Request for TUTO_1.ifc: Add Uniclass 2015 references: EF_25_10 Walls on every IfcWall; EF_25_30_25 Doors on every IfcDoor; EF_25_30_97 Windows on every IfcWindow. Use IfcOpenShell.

First a look at what the model holds.

```python
import ifcopenshell

model = ifcopenshell.open("TUTO_1.ifc")
print(model.schema)
print("classifications:", [c.Name for c in model.by_type("IfcClassification")])
for ifc_class in ("IfcDoor", "IfcRoof", "IfcStair", "IfcWall", "IfcWindow"):
    print(ifc_class, len(model.by_type(ifc_class)))
```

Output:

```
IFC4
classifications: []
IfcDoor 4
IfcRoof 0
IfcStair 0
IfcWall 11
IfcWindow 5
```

```python
import ifcopenshell
import ifcopenshell.api.classification

model = ifcopenshell.open("TUTO_1.ifc")

system = ifcopenshell.api.classification.add_classification(model, classification="Uniclass 2015")

codes = {
    "IfcWall": ("EF_25_10", "Walls"),
    "IfcDoor": ("EF_25_30_25", "Doors"),
    "IfcWindow": ("EF_25_30_97", "Windows"),
}
for ifc_class, (code, name) in codes.items():
    products = model.by_type(ifc_class)
    ifcopenshell.api.classification.add_reference(
        model, products=products, classification=system, identification=code, name=name
    )
    print(code, len(products))

model.write("TUTO_1_updated.ifc")
```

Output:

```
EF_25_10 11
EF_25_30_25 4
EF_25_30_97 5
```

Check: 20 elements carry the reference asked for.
